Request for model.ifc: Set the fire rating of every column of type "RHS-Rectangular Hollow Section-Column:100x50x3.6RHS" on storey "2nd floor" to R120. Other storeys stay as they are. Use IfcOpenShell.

First a look at what the model holds.

```python
import ifcopenshell
import ifcopenshell.util.element

model = ifcopenshell.open("model.ifc")
print(model.schema)
storey = next(s for s in model.by_type("IfcBuildingStorey") if s.Name == "2nd floor")
columns = [e for e in ifcopenshell.util.element.get_decomposition(storey) if e.is_a("IfcColumn")]
seen = {}
for e in columns:
    element_type = ifcopenshell.util.element.get_type(e)
    key = (element_type.Name if element_type != e and element_type else None, ifcopenshell.util.element.get_pset(e, "Pset_ColumnCommon", "FireRating"))
    seen[key] = seen.get(key, 0) + 1
for (name, value), count in sorted(seen.items(), key=str):
    print(count, "x", name, "|", value)
```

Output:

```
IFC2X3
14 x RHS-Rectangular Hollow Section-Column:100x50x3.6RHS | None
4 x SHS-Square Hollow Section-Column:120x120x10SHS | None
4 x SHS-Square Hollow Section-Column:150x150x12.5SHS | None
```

```python
import ifcopenshell
import ifcopenshell.api.pset
import ifcopenshell.util.element

model = ifcopenshell.open("model.ifc")

storey = next(s for s in model.by_type("IfcBuildingStorey") if s.Name == "2nd floor")
columns = [e for e in ifcopenshell.util.element.get_decomposition(storey) if e.is_a("IfcColumn")]

count = 0
for e in columns:
    element_type = ifcopenshell.util.element.get_type(e)
    if element_type in (None, e) or element_type.Name != "RHS-Rectangular Hollow Section-Column:100x50x3.6RHS":
        continue
    # add_pset returns the element's existing set when there is one.
    pset = ifcopenshell.api.pset.add_pset(model, product=e, name="Pset_ColumnCommon")
    ifcopenshell.api.pset.edit_pset(model, pset=pset, properties={"FireRating": "R120"})
    count += 1

print(count, "columns updated")

model.write("model_updated.ifc")
```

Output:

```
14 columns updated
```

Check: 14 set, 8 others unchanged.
